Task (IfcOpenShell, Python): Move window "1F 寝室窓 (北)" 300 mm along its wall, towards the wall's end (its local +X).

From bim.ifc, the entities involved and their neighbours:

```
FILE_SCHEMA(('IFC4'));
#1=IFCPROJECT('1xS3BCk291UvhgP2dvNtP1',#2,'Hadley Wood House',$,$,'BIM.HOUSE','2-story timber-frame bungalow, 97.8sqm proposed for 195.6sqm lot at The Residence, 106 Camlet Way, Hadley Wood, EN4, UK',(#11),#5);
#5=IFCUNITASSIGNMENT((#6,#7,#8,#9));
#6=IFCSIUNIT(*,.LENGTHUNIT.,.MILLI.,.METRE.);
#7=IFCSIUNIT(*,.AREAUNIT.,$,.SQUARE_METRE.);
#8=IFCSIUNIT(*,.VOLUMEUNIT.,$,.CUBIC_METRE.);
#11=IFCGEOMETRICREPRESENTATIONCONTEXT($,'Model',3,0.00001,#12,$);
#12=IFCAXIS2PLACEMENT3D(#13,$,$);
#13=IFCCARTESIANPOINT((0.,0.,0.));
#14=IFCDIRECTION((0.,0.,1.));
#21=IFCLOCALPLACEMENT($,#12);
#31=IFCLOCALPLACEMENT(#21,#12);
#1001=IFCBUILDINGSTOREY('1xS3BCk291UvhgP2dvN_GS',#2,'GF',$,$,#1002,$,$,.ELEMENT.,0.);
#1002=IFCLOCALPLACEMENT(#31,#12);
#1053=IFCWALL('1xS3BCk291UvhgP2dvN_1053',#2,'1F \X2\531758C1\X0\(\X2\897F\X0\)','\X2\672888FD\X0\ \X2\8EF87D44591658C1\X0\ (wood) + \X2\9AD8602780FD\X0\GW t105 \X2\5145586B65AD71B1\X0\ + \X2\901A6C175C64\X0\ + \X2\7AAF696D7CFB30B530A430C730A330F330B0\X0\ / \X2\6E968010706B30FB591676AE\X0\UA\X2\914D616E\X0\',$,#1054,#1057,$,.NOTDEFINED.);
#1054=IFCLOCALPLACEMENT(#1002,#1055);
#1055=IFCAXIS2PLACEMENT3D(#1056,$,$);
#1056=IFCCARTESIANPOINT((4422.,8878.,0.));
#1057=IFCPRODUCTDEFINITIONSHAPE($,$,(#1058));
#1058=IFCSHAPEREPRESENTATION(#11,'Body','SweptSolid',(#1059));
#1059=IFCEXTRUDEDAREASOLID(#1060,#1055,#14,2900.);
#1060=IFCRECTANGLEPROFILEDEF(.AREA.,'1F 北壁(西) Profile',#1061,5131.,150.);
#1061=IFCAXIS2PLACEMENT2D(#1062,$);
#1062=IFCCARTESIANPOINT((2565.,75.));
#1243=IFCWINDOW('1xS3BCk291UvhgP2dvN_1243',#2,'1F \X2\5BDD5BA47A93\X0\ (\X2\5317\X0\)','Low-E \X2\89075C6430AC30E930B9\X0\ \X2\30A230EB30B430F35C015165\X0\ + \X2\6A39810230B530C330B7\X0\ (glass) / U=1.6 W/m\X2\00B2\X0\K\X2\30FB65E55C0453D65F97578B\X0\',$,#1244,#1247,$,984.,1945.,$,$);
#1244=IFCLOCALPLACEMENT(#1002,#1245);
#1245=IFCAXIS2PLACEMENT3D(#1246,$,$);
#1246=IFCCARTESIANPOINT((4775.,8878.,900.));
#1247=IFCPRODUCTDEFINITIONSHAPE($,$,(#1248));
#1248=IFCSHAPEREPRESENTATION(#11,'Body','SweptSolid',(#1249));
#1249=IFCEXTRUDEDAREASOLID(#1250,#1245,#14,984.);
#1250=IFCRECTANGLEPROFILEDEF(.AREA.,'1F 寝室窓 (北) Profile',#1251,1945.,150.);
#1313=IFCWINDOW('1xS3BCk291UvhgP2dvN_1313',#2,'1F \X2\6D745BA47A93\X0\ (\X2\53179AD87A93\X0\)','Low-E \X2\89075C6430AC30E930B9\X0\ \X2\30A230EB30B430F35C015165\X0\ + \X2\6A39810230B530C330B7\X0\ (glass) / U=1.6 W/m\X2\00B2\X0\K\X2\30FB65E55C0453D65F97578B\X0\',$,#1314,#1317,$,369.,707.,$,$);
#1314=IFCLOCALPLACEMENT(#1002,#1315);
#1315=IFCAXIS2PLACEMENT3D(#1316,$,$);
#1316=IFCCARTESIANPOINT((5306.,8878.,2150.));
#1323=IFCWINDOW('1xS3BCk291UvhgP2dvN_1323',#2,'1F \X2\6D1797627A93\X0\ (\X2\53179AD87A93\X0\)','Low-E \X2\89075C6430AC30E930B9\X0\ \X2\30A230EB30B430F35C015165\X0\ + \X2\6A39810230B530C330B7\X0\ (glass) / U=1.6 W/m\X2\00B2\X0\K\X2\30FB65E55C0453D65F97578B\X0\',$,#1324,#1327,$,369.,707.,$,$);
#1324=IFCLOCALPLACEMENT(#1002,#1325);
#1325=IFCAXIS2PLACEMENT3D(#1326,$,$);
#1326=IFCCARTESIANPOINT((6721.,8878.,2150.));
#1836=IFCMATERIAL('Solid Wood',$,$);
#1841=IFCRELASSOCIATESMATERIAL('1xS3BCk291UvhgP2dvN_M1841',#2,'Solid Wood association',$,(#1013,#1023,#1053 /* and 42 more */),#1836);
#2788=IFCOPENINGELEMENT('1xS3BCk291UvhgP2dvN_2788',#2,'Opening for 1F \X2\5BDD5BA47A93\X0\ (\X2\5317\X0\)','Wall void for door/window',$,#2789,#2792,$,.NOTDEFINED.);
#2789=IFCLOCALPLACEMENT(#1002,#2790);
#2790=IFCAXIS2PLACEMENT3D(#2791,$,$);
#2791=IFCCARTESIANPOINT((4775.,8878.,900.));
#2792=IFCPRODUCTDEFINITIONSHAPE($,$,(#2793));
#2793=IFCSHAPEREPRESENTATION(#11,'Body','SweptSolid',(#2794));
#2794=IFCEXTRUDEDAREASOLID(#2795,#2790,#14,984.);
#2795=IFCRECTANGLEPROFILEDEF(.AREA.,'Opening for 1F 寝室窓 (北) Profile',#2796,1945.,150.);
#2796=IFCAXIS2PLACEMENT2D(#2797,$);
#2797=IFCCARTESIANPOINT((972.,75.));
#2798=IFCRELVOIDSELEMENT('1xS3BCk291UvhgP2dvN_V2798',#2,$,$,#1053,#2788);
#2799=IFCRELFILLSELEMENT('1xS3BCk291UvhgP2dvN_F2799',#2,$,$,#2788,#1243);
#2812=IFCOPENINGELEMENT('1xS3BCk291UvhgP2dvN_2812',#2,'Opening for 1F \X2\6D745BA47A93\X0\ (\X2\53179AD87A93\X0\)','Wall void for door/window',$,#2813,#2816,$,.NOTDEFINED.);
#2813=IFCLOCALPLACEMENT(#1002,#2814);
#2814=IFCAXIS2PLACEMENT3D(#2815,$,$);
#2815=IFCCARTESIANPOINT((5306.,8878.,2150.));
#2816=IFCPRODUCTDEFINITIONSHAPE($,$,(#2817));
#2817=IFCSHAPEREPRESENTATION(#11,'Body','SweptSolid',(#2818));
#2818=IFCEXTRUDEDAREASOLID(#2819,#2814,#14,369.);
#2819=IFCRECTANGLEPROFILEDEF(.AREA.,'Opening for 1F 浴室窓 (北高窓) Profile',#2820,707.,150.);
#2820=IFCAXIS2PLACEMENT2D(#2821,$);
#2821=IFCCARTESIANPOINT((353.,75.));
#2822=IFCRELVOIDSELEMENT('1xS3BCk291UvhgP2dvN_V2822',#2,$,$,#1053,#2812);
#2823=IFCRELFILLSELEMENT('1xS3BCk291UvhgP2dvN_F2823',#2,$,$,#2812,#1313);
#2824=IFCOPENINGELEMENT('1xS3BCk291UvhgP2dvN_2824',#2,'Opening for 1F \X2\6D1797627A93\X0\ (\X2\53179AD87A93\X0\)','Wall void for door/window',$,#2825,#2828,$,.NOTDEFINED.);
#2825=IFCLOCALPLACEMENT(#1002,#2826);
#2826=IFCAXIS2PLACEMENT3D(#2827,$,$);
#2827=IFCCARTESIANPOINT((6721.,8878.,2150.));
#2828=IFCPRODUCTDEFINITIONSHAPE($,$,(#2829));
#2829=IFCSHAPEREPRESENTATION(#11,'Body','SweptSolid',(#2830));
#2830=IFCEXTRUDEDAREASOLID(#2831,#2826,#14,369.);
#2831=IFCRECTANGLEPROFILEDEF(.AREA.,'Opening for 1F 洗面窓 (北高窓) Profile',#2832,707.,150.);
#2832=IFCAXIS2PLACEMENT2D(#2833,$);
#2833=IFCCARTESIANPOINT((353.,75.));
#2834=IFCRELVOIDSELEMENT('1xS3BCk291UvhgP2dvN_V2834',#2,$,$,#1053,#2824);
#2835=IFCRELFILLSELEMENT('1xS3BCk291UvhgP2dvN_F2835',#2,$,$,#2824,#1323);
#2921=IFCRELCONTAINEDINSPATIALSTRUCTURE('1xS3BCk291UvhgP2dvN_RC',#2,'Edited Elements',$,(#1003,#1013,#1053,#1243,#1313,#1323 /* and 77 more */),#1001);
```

```python
import ifcopenshell
import ifcopenshell.api.geometry
import ifcopenshell.util.placement

model = ifcopenshell.open("bim.ifc")

window = model.by_guid("1xS3BCk291UvhgP2dvN_1243")
opening = window.FillsVoids[0].RelatingOpeningElement
wall = opening.VoidsElements[0].RelatingBuildingElement

wall_matrix = ifcopenshell.util.placement.get_local_placement(wall.ObjectPlacement)
shift = wall_matrix[:3, 0] * 300.0
before = ifcopenshell.util.placement.get_local_placement(window.ObjectPlacement)[:3, 3].copy()

# The window is not placed relative to its opening, so move both.
for product in (opening, window):
    matrix = ifcopenshell.util.placement.get_local_placement(product.ObjectPlacement)
    matrix[:3, 3] += shift
    ifcopenshell.api.geometry.edit_object_placement(model, product=product, matrix=matrix, is_si=False)

after = ifcopenshell.util.placement.get_local_placement(window.ObjectPlacement)[:3, 3]
print("window moved by", (after - before).round(3) + 0.0)

model.write("bim_updated.ifc")
```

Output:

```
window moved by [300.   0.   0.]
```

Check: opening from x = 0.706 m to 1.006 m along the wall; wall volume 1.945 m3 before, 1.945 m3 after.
